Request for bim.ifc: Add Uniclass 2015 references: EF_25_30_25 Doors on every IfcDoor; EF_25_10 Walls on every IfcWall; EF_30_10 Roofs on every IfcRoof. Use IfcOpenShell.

First a look at what the model holds.

```python
import ifcopenshell

model = ifcopenshell.open("bim.ifc")
print(model.schema)
print("classifications:", [c.Name for c in model.by_type("IfcClassification")])
for ifc_class in ("IfcDoor", "IfcRoof", "IfcStair", "IfcWall", "IfcWindow"):
    print(ifc_class, len(model.by_type(ifc_class)))
```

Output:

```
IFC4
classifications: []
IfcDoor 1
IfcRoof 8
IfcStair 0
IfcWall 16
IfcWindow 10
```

```python
import ifcopenshell
import ifcopenshell.api.classification

model = ifcopenshell.open("bim.ifc")

system = ifcopenshell.api.classification.add_classification(model, classification="Uniclass 2015")

codes = {
    "IfcDoor": ("EF_25_30_25", "Doors"),
    "IfcWall": ("EF_25_10", "Walls"),
    "IfcRoof": ("EF_30_10", "Roofs"),
}
for ifc_class, (code, name) in codes.items():
    products = model.by_type(ifc_class)
    ifcopenshell.api.classification.add_reference(
        model, products=products, classification=system, identification=code, name=name
    )
    print(code, len(products))

model.write("bim-out.ifc")
```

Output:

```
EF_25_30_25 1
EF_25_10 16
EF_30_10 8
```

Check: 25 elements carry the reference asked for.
